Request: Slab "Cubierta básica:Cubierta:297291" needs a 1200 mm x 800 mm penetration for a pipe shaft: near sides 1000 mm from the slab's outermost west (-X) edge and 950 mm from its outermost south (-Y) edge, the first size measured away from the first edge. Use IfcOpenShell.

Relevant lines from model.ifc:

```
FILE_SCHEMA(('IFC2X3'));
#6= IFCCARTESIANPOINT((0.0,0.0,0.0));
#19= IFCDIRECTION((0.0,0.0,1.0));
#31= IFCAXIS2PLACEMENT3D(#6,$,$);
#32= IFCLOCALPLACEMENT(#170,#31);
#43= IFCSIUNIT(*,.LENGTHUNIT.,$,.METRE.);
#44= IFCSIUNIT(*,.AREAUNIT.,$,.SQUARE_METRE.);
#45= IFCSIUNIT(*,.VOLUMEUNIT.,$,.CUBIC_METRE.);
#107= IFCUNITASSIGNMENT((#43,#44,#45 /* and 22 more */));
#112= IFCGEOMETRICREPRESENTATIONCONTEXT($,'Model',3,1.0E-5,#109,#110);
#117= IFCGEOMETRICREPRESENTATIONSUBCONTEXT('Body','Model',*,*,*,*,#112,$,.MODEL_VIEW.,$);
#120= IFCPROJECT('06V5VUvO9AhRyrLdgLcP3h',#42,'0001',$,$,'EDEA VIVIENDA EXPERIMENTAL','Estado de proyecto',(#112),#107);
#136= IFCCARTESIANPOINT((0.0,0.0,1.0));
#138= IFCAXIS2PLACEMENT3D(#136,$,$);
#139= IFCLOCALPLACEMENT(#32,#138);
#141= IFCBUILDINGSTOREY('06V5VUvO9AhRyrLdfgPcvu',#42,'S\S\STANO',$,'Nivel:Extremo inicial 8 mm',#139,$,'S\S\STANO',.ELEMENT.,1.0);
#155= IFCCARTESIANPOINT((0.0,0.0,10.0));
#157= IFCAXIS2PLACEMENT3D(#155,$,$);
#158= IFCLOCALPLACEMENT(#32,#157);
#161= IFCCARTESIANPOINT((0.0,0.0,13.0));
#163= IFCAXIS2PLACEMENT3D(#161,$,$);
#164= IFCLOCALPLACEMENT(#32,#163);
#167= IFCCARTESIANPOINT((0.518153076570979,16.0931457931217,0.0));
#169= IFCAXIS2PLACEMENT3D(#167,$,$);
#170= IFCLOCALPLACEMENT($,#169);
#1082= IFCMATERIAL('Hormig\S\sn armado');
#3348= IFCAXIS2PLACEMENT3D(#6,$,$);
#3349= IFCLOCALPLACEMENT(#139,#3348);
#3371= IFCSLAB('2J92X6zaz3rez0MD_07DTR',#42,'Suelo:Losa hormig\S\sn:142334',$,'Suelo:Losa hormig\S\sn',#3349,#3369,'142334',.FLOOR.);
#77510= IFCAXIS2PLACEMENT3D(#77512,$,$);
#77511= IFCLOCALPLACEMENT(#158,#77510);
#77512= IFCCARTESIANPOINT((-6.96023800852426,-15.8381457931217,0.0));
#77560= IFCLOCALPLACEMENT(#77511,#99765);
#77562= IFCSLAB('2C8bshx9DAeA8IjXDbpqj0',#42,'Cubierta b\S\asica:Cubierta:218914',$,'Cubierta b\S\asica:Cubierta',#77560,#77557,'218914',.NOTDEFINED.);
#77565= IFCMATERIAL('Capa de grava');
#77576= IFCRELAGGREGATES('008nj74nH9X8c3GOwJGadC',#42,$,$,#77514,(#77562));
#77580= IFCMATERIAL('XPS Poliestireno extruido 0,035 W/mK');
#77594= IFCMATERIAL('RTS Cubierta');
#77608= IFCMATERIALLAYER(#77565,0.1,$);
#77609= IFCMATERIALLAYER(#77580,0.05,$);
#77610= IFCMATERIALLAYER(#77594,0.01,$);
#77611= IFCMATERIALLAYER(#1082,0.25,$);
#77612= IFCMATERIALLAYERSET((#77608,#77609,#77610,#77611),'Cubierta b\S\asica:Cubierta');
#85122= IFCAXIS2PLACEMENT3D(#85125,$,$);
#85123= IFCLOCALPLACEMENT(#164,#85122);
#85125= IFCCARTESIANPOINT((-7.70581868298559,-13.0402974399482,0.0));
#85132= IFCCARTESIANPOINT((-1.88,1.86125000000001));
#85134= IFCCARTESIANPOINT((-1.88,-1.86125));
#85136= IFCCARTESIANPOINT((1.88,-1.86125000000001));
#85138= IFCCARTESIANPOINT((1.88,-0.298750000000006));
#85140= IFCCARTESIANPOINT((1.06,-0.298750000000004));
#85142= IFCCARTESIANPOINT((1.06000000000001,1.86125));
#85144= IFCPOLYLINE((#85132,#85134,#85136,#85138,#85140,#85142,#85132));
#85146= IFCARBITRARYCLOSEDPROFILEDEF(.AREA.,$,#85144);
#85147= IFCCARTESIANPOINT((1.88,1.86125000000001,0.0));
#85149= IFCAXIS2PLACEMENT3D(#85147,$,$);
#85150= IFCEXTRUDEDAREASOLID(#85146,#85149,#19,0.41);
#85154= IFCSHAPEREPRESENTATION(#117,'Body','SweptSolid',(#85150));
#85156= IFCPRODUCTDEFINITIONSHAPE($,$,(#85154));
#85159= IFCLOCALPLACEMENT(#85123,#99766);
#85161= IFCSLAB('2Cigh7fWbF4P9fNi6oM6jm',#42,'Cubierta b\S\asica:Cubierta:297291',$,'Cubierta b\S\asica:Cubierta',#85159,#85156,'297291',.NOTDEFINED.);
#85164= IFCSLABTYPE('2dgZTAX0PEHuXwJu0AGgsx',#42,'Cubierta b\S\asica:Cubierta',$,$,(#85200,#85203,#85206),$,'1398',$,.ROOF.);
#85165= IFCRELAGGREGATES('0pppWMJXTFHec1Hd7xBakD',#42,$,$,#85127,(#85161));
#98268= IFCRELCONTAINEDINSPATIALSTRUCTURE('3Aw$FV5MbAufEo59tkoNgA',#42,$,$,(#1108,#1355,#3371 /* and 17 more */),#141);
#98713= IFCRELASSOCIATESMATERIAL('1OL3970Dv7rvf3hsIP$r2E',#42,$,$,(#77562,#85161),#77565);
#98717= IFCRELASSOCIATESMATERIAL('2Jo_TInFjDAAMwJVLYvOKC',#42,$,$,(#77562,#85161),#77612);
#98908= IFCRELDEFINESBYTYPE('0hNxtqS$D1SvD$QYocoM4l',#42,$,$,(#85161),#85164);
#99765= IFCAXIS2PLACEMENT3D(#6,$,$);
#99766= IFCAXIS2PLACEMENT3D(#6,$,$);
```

```python
import numpy as np
import ifcopenshell
import ifcopenshell.api.feature
import ifcopenshell.api.geometry
import ifcopenshell.api.root
import ifcopenshell.geom
import ifcopenshell.util.placement
import ifcopenshell.util.representation
import ifcopenshell.util.shape
import ifcopenshell.util.unit

model = ifcopenshell.open("model.ifc")
unit_scale = ifcopenshell.util.unit.calculate_unit_scale(model)
settings = ifcopenshell.geom.settings()


def volume(element):
    """Net volume in cubic metres, openings subtracted."""
    shape = ifcopenshell.geom.create_shape(settings, element)
    return ifcopenshell.util.shape.get_volume(shape.geometry)


slab = model.by_guid("2Cigh7fWbF4P9fNi6oM6jm")
before = volume(slab)

# Extent in the slab's own axes, in metres. The edges named are its -X and -Y sides.
slab_shape = ifcopenshell.geom.create_shape(settings, slab)
vertices = ifcopenshell.util.shape.get_vertices(slab_shape.geometry)
x_min, y_min, bottom = vertices.min(axis=0)
top = vertices[:, 2].max()

opening = ifcopenshell.api.root.create_entity(model, ifc_class="IfcOpeningElement", name="Pipe shaft opening")
context = ifcopenshell.util.representation.get_context(model, "Model", "Body", "MODEL_VIEW")
width, depth = 1.2, 0.8
outline = [(0.0, 0.0), (width, 0.0), (width, depth), (0.0, depth), (0.0, 0.0)]
# Overshoot both faces by 50 mm so the cut is clean.
shape = ifcopenshell.api.geometry.add_slab_representation(
    model, context=context, depth=top - bottom + 0.1, polyline=outline
)
ifcopenshell.api.geometry.assign_representation(model, product=opening, representation=shape)

matrix = ifcopenshell.util.placement.get_local_placement(slab.ObjectPlacement)
matrix[:, 3] = matrix @ np.append(np.array([x_min + 1, y_min + 0.95, bottom - 0.05]) / unit_scale, 1.0)
ifcopenshell.api.geometry.edit_object_placement(model, product=opening, matrix=matrix, is_si=False)
ifcopenshell.api.feature.add_feature(model, feature=opening, element=slab)

after = volume(slab)

print(f"slab volume {before:.3f} -> {after:.3f} m3")

model.write("model_rev.ifc")
```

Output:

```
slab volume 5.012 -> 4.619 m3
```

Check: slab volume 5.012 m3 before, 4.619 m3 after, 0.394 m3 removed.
